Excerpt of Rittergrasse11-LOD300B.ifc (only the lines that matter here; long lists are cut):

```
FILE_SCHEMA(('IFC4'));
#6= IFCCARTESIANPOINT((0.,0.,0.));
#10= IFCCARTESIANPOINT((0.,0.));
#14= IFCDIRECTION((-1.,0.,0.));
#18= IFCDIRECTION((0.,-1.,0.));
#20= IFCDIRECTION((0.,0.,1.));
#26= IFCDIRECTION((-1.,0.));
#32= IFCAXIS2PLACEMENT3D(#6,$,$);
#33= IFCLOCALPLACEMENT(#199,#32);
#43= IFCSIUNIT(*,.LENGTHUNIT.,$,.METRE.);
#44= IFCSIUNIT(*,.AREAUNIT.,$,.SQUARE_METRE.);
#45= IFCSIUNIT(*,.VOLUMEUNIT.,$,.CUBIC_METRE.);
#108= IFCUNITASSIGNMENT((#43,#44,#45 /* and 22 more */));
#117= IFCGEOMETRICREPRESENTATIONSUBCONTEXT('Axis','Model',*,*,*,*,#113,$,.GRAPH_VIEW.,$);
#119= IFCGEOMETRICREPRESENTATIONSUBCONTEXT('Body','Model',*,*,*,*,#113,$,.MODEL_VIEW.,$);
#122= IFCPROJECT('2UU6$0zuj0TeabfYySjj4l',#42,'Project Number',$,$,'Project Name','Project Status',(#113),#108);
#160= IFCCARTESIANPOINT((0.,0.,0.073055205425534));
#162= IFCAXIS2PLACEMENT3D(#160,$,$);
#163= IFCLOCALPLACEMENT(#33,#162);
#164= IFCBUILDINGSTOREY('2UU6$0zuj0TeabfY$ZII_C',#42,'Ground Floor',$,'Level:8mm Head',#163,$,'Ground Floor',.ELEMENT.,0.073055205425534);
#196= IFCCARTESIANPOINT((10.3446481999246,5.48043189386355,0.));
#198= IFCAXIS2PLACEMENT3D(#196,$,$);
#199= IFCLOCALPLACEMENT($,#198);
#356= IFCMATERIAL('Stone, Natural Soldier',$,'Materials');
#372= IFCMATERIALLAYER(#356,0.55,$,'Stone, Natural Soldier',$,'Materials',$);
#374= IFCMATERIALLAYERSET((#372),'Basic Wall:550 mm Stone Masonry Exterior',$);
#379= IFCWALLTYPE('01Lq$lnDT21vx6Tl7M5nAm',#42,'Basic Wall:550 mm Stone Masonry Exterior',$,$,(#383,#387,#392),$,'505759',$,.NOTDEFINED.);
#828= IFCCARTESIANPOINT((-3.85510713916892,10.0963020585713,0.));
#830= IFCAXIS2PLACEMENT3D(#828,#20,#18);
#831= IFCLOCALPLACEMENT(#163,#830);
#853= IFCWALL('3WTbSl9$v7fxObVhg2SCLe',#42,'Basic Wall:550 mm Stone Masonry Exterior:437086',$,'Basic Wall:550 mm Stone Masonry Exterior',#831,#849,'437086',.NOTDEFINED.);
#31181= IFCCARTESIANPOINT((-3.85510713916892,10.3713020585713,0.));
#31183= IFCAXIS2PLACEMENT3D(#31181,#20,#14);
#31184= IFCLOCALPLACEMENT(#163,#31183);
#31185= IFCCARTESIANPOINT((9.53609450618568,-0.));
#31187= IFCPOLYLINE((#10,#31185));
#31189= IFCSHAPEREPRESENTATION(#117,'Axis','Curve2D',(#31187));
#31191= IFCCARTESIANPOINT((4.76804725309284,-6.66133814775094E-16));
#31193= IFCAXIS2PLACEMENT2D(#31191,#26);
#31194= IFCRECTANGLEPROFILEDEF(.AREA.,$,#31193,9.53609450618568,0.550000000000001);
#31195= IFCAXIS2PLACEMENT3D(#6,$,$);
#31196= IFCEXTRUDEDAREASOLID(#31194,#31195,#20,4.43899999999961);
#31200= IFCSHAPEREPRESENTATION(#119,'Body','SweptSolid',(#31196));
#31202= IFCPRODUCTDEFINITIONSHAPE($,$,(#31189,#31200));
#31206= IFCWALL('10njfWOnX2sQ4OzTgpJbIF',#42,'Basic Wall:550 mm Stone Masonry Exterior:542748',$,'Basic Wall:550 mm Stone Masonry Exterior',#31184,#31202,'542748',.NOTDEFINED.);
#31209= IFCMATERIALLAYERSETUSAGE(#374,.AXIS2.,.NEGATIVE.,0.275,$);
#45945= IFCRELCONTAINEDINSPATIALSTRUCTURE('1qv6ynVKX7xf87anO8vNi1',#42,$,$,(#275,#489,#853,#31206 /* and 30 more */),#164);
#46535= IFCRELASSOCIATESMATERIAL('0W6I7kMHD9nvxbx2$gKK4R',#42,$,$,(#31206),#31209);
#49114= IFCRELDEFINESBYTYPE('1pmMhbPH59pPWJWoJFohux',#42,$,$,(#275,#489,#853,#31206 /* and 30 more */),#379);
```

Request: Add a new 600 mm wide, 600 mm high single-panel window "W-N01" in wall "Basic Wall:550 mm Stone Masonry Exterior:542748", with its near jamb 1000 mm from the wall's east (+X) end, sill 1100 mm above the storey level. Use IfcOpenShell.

```python
import numpy as np
import ifcopenshell
import ifcopenshell.api.feature
import ifcopenshell.api.geometry
import ifcopenshell.api.root
import ifcopenshell.api.spatial
import ifcopenshell.geom
import ifcopenshell.util.element
import ifcopenshell.util.placement
import ifcopenshell.util.representation
import ifcopenshell.util.shape
import ifcopenshell.util.unit

model = ifcopenshell.open("Rittergrasse11-LOD300B.ifc")
unit_scale = ifcopenshell.util.unit.calculate_unit_scale(model)
settings = ifcopenshell.geom.settings()


def volume(element):
    """Net volume in cubic metres, openings subtracted."""
    shape = ifcopenshell.geom.create_shape(settings, element)
    return ifcopenshell.util.shape.get_volume(shape.geometry)


wall = model.by_id(31206)
storey = ifcopenshell.util.element.get_container(wall, ifc_class="IfcBuildingStorey")
context = ifcopenshell.util.representation.get_context(model, "Model", "Body", "MODEL_VIEW")
before = volume(wall)

width, height, from_end, sill = 0.6, 0.6, 1, 1.1  # metres

# The wall runs along its own X axis, and the end named is its -X end.
wall_shape = ifcopenshell.geom.create_shape(settings, wall)
x, y, z = ifcopenshell.util.shape.get_vertices(wall_shape.geometry).T
start = x.min() + from_end
face, thickness = float(y.min()), float(y.max() - y.min())
wall_matrix = ifcopenshell.util.placement.get_local_placement(wall.ObjectPlacement)
level = ifcopenshell.util.placement.get_local_placement(storey.ObjectPlacement)[2, 3]


def in_wall(x, y):
    """Placement at x, y metres in the wall's axes, at sill height."""
    matrix = wall_matrix.copy()
    matrix[:, 3] = wall_matrix @ np.array([x / unit_scale, y / unit_scale, 0.0, 1.0])
    matrix[2, 3] = level + sill / unit_scale
    return matrix


# Opening: a box that overshoots both wall faces by 50 mm.
opening = ifcopenshell.api.root.create_entity(model, ifc_class="IfcOpeningElement", predefined_type="OPENING")
box = ifcopenshell.api.geometry.add_wall_representation(
    model, context=context, length=width, height=height, thickness=thickness + 0.1
)
ifcopenshell.api.geometry.assign_representation(model, product=opening, representation=box)
ifcopenshell.api.geometry.edit_object_placement(model, product=opening, matrix=in_wall(start, face - 0.05), is_si=False)
ifcopenshell.api.feature.add_feature(model, feature=opening, element=wall)

window = ifcopenshell.api.root.create_entity(model, ifc_class="IfcWindow", name="W-N01", predefined_type="WINDOW")
window.OverallWidth, window.OverallHeight = width / unit_scale, height / unit_scale
window.PartitioningType = "SINGLE_PANEL"
body = ifcopenshell.api.geometry.add_window_representation(
    model,
    context=context,
    overall_width=window.OverallWidth,
    overall_height=window.OverallHeight,
    partition_type="SINGLE_PANEL",
)
ifcopenshell.api.geometry.assign_representation(model, product=window, representation=body)
ifcopenshell.api.spatial.assign_container(model, products=[window], relating_structure=storey)
ifcopenshell.api.feature.add_filling(model, opening=opening, element=window)

# Centre the window in the wall's thickness.
ifcopenshell.api.geometry.edit_object_placement(model, product=window, matrix=in_wall(start, face), is_si=False)
window_shape = ifcopenshell.geom.create_shape(settings, window)
depth = ifcopenshell.util.shape.get_vertices(window_shape.geometry)[:, 1]
offset = face + thickness / 2 - (depth.min() + depth.max()) / 2
ifcopenshell.api.geometry.edit_object_placement(model, product=window, matrix=in_wall(start, offset), is_si=False)

after = volume(wall)

print(f"wall volume {before:.3f} -> {after:.3f} m3")

model.write("Rittergrasse11-LOD300B_v2.ifc")
```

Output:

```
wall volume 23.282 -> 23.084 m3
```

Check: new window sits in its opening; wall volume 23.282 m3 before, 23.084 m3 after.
